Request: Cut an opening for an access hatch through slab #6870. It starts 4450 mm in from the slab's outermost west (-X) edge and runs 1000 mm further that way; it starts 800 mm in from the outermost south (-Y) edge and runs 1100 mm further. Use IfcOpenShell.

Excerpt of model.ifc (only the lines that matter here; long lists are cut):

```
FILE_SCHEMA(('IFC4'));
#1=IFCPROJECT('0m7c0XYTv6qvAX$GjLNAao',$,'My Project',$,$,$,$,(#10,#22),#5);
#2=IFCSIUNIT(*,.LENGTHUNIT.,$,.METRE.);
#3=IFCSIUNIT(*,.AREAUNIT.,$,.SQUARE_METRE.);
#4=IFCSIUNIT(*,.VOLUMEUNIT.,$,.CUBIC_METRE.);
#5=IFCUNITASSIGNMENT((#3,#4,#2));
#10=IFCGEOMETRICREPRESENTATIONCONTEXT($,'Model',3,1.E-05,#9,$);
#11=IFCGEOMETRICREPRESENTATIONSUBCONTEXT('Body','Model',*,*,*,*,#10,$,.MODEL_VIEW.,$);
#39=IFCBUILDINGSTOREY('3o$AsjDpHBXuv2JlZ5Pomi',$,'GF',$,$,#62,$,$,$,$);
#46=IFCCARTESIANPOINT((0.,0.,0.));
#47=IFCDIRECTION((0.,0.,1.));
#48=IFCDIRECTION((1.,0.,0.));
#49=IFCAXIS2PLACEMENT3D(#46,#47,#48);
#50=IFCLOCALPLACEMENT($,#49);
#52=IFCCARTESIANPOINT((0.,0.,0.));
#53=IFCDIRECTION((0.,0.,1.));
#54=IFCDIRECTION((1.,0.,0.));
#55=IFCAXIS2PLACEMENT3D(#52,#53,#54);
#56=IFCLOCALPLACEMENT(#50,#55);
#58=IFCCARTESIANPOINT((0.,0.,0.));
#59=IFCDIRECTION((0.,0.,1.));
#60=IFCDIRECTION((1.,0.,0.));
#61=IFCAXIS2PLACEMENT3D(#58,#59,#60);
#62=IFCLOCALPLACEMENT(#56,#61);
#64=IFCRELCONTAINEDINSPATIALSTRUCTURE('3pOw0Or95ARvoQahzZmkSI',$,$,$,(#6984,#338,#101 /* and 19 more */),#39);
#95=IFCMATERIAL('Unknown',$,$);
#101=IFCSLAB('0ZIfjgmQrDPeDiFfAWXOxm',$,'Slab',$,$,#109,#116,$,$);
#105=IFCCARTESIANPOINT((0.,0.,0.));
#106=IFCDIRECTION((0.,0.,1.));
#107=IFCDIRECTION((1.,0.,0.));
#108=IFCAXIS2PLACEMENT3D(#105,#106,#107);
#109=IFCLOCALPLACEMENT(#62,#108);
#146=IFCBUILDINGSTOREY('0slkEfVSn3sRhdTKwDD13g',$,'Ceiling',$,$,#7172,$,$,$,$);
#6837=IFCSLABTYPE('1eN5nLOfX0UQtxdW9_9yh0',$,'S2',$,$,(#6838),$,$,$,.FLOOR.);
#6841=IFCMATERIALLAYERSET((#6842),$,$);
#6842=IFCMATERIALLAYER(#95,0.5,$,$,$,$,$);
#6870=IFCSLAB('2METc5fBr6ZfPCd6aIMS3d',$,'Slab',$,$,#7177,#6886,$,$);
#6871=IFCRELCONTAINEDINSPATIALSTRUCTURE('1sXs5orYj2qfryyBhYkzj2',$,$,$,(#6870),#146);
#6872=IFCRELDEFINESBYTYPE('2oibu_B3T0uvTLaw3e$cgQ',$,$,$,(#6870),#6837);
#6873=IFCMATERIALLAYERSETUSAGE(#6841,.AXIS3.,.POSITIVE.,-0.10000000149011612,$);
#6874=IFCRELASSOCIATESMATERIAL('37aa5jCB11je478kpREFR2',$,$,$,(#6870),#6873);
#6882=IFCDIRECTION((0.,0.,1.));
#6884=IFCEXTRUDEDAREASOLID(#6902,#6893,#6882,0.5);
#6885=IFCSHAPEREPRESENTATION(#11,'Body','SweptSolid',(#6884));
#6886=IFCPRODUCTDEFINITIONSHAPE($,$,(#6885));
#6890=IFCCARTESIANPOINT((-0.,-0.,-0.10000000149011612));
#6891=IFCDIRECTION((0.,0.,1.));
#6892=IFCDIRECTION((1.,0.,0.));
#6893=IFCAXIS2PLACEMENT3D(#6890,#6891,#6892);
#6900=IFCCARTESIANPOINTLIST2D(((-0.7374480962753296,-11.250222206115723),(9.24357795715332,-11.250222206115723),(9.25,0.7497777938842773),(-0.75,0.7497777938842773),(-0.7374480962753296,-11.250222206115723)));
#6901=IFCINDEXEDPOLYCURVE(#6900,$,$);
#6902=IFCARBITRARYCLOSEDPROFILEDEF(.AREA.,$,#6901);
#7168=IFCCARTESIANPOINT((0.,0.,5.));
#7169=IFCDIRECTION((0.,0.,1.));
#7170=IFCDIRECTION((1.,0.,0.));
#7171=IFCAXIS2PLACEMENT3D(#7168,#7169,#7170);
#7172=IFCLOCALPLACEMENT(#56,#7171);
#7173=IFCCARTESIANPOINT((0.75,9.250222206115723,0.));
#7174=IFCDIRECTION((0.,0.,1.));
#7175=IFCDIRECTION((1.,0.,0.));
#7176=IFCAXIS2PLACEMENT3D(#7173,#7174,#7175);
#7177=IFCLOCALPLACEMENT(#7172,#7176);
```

```python
import numpy as np
import ifcopenshell
import ifcopenshell.api.feature
import ifcopenshell.api.geometry
import ifcopenshell.api.root
import ifcopenshell.geom
import ifcopenshell.util.placement
import ifcopenshell.util.representation
import ifcopenshell.util.shape
import ifcopenshell.util.unit

model = ifcopenshell.open("model.ifc")
unit_scale = ifcopenshell.util.unit.calculate_unit_scale(model)
settings = ifcopenshell.geom.settings()


def volume(element):
    """Net volume in cubic metres, openings subtracted."""
    shape = ifcopenshell.geom.create_shape(settings, element)
    return ifcopenshell.util.shape.get_volume(shape.geometry)


slab = model.by_guid("2METc5fBr6ZfPCd6aIMS3d")
before = volume(slab)

# Extent in the slab's own axes, in metres. The edges named are its -X and -Y sides.
slab_shape = ifcopenshell.geom.create_shape(settings, slab)
vertices = ifcopenshell.util.shape.get_vertices(slab_shape.geometry)
x_min, y_min, bottom = vertices.min(axis=0)
top = vertices[:, 2].max()

opening = ifcopenshell.api.root.create_entity(model, ifc_class="IfcOpeningElement", name="Access hatch opening", predefined_type="OPENING")
context = ifcopenshell.util.representation.get_context(model, "Model", "Body", "MODEL_VIEW")
width, depth = 1, 1.1
outline = [(0.0, 0.0), (width, 0.0), (width, depth), (0.0, depth), (0.0, 0.0)]
# Overshoot both faces by 50 mm so the cut is clean.
shape = ifcopenshell.api.geometry.add_slab_representation(
    model, context=context, depth=top - bottom + 0.1, polyline=outline
)
ifcopenshell.api.geometry.assign_representation(model, product=opening, representation=shape)

matrix = ifcopenshell.util.placement.get_local_placement(slab.ObjectPlacement)
matrix[:, 3] = matrix @ np.append(np.array([x_min + 4.45, y_min + 0.8, bottom - 0.05]) / unit_scale, 1.0)
ifcopenshell.api.geometry.edit_object_placement(model, product=opening, matrix=matrix, is_si=False)
ifcopenshell.api.feature.add_feature(model, feature=opening, element=slab)

after = volume(slab)

print(f"slab volume {before:.3f} -> {after:.3f} m3")

model.write("model_edited.ifc")
```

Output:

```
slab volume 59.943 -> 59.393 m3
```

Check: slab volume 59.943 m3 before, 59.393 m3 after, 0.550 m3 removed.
